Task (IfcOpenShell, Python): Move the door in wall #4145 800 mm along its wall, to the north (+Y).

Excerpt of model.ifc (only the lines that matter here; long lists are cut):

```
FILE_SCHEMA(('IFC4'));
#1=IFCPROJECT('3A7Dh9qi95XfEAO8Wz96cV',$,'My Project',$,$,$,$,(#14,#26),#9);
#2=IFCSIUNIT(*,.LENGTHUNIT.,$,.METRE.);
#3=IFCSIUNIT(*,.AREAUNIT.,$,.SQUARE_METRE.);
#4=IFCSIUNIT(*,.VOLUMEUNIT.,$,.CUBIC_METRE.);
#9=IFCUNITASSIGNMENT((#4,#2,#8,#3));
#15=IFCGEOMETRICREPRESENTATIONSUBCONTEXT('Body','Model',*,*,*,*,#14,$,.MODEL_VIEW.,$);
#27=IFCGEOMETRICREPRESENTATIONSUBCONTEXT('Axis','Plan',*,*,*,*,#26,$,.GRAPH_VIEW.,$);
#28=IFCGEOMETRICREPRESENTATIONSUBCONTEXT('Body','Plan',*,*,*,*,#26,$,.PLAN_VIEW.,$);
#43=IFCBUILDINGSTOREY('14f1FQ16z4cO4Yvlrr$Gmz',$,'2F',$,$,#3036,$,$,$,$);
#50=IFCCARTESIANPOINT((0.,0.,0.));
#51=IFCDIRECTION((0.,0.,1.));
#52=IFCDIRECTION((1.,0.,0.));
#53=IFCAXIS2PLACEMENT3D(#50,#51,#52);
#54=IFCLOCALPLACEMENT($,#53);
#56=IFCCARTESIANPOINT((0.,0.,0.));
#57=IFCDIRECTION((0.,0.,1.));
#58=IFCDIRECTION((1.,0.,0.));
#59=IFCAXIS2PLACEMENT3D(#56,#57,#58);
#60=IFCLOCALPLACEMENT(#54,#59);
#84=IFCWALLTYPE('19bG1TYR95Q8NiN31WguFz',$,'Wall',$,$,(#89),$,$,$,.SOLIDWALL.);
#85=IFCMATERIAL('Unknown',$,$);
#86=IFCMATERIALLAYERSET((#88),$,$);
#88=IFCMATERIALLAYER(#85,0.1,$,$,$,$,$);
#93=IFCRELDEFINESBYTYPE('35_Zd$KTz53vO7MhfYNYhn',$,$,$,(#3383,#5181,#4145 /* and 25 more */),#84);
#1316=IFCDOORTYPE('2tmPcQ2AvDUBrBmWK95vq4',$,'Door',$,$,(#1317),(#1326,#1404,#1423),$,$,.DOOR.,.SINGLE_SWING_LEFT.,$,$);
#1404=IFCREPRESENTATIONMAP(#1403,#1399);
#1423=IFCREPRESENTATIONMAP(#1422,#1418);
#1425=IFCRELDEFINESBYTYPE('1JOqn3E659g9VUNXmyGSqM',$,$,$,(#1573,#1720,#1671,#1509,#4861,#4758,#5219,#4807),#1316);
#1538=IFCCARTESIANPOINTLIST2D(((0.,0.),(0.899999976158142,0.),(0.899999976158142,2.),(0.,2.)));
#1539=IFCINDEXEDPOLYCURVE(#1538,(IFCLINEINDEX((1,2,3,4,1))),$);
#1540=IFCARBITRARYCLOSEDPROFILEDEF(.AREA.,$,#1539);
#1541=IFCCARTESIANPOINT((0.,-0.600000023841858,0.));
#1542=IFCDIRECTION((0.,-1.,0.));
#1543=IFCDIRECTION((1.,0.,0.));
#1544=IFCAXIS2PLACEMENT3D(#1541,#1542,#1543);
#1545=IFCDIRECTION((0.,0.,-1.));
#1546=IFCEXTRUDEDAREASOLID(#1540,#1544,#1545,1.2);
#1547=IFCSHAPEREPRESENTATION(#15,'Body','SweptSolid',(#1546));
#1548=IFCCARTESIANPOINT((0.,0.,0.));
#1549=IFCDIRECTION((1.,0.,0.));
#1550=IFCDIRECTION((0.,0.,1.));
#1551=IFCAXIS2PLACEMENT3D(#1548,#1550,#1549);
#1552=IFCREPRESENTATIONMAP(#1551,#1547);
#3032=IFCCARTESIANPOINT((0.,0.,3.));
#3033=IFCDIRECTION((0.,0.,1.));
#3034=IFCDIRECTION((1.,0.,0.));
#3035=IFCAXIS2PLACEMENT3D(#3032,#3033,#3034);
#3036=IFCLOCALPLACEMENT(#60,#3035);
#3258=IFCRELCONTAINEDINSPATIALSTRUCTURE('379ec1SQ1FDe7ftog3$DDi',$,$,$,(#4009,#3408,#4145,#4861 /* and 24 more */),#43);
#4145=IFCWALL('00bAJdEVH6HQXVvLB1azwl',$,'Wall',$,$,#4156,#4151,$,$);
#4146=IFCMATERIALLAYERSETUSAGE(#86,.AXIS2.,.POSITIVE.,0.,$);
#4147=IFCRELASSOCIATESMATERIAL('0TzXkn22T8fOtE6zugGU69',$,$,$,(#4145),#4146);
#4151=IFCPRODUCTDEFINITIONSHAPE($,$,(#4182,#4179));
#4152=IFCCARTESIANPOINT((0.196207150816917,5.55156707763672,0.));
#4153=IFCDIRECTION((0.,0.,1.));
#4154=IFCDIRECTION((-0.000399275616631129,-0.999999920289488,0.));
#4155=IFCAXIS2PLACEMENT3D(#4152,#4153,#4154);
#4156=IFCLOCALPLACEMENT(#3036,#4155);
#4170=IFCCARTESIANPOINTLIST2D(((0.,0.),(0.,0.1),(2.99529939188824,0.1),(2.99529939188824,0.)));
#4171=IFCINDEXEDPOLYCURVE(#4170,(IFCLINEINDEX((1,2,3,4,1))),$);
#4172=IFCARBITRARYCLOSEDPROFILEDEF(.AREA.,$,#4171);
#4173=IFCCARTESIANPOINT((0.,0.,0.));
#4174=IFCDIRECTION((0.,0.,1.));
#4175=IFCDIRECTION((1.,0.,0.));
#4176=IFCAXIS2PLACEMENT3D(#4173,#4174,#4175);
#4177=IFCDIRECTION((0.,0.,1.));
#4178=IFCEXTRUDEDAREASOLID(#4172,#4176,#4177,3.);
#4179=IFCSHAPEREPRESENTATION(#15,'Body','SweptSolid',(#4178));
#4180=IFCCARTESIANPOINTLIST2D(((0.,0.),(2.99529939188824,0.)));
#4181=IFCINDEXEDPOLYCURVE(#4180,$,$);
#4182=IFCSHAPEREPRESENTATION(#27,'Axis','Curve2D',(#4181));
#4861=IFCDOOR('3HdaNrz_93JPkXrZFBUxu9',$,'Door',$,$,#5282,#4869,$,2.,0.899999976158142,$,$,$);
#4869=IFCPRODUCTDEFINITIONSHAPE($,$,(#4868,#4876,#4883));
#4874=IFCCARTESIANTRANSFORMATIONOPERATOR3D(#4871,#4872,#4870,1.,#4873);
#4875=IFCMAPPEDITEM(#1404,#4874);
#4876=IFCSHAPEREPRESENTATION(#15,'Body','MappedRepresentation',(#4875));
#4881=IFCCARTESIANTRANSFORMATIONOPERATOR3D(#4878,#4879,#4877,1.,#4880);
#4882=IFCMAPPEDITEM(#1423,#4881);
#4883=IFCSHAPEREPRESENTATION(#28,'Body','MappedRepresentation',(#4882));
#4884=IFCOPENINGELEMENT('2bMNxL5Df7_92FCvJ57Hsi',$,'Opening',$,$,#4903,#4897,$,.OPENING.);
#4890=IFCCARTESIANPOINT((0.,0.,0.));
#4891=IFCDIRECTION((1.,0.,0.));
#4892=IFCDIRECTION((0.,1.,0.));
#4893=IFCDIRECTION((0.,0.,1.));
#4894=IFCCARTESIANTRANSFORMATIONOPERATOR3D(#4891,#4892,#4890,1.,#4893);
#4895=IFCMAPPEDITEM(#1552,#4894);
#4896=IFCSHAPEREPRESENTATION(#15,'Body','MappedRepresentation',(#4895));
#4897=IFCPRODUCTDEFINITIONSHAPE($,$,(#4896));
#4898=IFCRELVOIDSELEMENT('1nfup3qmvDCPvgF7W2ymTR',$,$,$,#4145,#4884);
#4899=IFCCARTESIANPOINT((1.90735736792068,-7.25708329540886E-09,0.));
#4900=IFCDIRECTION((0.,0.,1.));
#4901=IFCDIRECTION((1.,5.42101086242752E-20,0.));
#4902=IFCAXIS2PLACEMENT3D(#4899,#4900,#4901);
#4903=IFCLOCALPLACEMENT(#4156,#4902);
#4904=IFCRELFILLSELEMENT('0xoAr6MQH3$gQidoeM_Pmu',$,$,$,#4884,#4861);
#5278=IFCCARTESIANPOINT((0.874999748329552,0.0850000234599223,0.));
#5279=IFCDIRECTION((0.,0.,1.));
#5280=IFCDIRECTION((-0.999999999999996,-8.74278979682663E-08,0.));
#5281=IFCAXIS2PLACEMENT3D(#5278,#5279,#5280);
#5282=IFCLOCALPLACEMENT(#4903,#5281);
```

```python
import ifcopenshell
import ifcopenshell.api.geometry
import ifcopenshell.util.placement
import ifcopenshell.util.unit

model = ifcopenshell.open("model.ifc")
unit_scale = ifcopenshell.util.unit.calculate_unit_scale(model)

door = model.by_id(4861)
opening = door.FillsVoids[0].RelatingOpeningElement
wall = opening.VoidsElements[0].RelatingBuildingElement

wall_matrix = ifcopenshell.util.placement.get_local_placement(wall.ObjectPlacement)
shift = wall_matrix[:3, 0] * -0.8 / unit_scale
before = ifcopenshell.util.placement.get_local_placement(door.ObjectPlacement)[:3, 3].copy()

# The door is placed relative to its opening, so it follows when the opening moves.
matrix = ifcopenshell.util.placement.get_local_placement(opening.ObjectPlacement)
matrix[:3, 3] += shift
ifcopenshell.api.geometry.edit_object_placement(
    model, product=opening, matrix=matrix, is_si=False, should_transform_children=True
)

after = ifcopenshell.util.placement.get_local_placement(door.ObjectPlacement)[:3, 3]
print("door moved by", (after - before).round(3) + 0.0)

model.write("model-out.ifc")
```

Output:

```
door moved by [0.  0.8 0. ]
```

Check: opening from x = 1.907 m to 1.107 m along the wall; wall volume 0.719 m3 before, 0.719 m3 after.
